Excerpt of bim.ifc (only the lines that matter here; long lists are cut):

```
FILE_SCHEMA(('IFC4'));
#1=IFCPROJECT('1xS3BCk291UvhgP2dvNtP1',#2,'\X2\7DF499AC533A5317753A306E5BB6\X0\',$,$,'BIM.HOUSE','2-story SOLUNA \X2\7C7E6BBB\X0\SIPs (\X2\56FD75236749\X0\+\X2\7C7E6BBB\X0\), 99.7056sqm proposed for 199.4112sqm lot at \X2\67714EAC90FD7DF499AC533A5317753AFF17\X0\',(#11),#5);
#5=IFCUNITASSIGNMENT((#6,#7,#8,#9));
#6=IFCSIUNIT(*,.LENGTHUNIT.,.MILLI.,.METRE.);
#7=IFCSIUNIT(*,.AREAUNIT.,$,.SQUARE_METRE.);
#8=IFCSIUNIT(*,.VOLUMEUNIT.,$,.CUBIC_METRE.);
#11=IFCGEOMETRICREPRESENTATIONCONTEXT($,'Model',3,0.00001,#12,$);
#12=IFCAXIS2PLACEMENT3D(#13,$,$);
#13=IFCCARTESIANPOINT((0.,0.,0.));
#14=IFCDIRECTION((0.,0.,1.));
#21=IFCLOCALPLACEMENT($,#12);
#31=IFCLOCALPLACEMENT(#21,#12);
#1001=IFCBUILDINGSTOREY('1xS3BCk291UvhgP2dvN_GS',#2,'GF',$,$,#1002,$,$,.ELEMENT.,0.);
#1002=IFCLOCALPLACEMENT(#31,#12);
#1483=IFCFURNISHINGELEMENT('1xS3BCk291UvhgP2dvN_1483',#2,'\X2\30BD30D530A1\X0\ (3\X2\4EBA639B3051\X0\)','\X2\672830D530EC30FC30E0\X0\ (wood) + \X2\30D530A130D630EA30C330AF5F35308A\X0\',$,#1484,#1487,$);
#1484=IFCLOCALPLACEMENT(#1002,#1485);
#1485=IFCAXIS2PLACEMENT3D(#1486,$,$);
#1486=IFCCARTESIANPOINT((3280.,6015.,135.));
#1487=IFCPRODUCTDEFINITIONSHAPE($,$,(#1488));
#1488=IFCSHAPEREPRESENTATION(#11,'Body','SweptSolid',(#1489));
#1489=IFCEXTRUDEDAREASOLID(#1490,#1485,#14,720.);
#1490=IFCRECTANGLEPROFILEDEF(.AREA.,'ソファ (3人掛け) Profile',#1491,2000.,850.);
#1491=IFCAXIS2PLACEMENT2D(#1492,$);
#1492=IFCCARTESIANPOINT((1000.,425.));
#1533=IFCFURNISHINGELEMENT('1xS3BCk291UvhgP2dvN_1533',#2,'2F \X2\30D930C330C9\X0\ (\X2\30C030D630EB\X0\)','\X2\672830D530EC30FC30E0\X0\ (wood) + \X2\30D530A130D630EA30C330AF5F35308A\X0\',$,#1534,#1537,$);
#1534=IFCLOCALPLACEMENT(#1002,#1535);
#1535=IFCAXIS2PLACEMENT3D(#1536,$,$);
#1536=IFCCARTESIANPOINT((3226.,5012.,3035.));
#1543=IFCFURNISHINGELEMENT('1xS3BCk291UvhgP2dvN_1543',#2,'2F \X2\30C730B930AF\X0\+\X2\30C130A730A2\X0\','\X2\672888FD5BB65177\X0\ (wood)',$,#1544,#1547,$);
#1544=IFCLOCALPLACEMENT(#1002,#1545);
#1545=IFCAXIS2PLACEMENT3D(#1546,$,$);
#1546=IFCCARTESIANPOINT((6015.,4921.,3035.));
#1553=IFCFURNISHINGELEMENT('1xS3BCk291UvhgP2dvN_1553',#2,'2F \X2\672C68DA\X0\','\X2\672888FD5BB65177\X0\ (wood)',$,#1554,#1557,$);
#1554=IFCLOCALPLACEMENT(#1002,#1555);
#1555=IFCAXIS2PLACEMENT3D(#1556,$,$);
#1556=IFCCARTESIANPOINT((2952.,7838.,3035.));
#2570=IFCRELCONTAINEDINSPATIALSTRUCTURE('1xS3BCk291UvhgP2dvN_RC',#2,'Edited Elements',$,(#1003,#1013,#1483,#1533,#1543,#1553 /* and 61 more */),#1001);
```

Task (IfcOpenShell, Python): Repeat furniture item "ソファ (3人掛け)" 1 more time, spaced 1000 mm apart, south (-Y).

```python
import numpy as np
import ifcopenshell
import ifcopenshell.api.geometry
import ifcopenshell.api.root
import ifcopenshell.util.element
import ifcopenshell.util.placement

model = ifcopenshell.open("bim.ifc")


def reuse_history(source, copy):
    """copy_class also copies each property set's owner history, people and application; keep the originals."""
    for rel in copy.IsDefinedBy:
        if rel.is_a("IfcRelDefinesByProperties") and (history := rel.RelatingPropertyDefinition.OwnerHistory):
            rel.RelatingPropertyDefinition.OwnerHistory = source.OwnerHistory
            ifcopenshell.util.element.remove_deep2(model, history)


source = model.by_guid("1xS3BCk291UvhgP2dvN_1483")
base = ifcopenshell.util.placement.get_local_placement(source.ObjectPlacement)
step = np.array([0.0, -1.0, 0.0]) * 1000.0

for i in range(1, 2):
    copy = ifcopenshell.api.root.copy_class(model, product=source)
    copy.Representation = ifcopenshell.util.element.copy_deep(
        model, source.Representation, exclude=["IfcGeometricRepresentationContext", "IfcRepresentationMap"]
    )
    reuse_history(source, copy)
    matrix = base.copy()
    matrix[:3, 3] += i * step
    print("added at", matrix[:3, 3].round(3) + 0.0)
    ifcopenshell.api.geometry.edit_object_placement(model, product=copy, matrix=matrix, is_si=False)

model.write("bim-out.ifc")
```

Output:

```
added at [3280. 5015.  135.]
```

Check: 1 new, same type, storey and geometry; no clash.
